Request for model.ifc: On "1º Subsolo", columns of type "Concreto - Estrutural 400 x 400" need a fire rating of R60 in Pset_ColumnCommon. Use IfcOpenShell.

First a look at what the model holds.

```python
import ifcopenshell
import ifcopenshell.util.element

model = ifcopenshell.open("model.ifc")
print(model.schema)
storey = next(s for s in model.by_type("IfcBuildingStorey") if s.Name == "1º Subsolo")
columns = [e for e in ifcopenshell.util.element.get_decomposition(storey) if e.is_a("IfcColumn")]
seen = {}
for e in columns:
    element_type = ifcopenshell.util.element.get_type(e)
    key = (element_type.Name if element_type != e and element_type else None, ifcopenshell.util.element.get_pset(e, "Pset_ColumnCommon", "FireRating"))
    seen[key] = seen.get(key, 0) + 1
for (name, value), count in sorted(seen.items(), key=str):
    print(count, "x", name, "|", value)
```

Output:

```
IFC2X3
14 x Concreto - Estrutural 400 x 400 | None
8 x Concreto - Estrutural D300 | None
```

```python
import ifcopenshell
import ifcopenshell.api.pset
import ifcopenshell.util.element

model = ifcopenshell.open("model.ifc")

storey = next(s for s in model.by_type("IfcBuildingStorey") if s.Name == "1º Subsolo")
columns = [e for e in ifcopenshell.util.element.get_decomposition(storey) if e.is_a("IfcColumn")]

count = 0
for e in columns:
    element_type = ifcopenshell.util.element.get_type(e)
    if element_type in (None, e) or element_type.Name != "Concreto - Estrutural 400 x 400":
        continue
    # add_pset returns the element's existing set when there is one.
    pset = ifcopenshell.api.pset.add_pset(model, product=e, name="Pset_ColumnCommon")
    ifcopenshell.api.pset.edit_pset(model, pset=pset, properties={"FireRating": "R60"})
    count += 1

print(count, "columns updated")

model.write("model_rev.ifc")
```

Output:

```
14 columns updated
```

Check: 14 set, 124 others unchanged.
